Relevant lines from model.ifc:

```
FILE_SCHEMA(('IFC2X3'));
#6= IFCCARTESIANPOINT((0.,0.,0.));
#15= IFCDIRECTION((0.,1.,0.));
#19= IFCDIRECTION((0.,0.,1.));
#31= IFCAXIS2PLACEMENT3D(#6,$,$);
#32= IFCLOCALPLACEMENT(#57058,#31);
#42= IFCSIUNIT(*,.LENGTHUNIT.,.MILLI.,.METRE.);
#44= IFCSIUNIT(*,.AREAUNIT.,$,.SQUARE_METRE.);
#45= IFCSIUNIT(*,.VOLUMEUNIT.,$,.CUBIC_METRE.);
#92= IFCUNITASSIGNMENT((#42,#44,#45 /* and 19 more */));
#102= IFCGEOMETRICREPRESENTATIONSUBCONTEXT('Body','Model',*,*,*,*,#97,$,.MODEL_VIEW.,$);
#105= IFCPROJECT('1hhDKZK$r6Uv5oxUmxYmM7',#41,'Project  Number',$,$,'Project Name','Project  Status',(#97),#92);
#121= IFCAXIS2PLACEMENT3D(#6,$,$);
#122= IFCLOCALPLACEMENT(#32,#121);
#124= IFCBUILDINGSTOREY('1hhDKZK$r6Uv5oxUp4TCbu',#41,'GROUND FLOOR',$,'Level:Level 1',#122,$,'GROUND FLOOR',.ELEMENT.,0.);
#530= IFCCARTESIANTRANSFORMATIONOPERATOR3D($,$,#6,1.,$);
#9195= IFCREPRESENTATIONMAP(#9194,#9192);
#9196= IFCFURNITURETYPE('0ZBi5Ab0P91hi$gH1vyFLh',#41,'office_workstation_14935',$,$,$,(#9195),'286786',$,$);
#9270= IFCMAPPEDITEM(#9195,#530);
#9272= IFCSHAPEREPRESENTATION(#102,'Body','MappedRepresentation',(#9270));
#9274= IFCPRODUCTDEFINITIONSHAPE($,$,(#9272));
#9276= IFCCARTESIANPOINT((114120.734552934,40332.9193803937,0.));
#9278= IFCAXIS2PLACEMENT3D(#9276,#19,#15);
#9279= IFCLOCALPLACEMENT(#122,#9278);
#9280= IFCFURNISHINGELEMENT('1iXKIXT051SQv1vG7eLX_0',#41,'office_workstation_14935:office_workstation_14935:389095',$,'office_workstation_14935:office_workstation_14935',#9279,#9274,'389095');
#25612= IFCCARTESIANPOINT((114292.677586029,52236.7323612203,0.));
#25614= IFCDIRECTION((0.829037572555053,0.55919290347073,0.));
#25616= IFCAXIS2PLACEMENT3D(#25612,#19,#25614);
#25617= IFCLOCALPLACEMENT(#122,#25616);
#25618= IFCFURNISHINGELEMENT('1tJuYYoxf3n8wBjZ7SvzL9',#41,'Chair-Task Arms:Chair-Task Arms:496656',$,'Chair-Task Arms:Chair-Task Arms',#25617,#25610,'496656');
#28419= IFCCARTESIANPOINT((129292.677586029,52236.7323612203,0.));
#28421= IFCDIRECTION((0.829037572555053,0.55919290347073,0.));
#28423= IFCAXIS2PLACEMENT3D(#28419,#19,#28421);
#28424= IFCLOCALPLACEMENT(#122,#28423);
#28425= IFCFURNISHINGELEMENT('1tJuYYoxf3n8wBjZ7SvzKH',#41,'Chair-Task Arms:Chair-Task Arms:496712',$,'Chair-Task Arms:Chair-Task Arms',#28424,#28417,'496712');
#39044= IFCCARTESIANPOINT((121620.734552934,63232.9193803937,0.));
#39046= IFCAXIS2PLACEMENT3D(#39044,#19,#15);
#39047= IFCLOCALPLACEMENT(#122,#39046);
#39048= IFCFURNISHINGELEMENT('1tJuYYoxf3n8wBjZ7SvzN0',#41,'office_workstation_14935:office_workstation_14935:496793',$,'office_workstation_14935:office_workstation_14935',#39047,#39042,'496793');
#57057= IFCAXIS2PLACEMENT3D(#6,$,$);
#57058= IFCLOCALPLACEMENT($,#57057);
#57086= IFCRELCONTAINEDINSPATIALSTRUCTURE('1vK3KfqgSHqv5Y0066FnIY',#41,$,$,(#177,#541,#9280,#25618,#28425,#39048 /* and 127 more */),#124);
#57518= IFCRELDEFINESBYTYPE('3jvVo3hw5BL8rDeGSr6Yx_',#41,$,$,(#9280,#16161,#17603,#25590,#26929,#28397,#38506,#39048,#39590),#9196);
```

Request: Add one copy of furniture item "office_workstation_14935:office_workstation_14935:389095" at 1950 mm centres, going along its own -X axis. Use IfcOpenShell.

```python
import ifcopenshell
import ifcopenshell.api.geometry
import ifcopenshell.api.root
import ifcopenshell.util.element
import ifcopenshell.util.placement
import ifcopenshell.util.unit

model = ifcopenshell.open("model.ifc")
unit_scale = ifcopenshell.util.unit.calculate_unit_scale(model)


def reuse_history(source, copy):
    """copy_class also copies each property set's owner history, people and application; keep the originals."""
    for rel in copy.IsDefinedBy:
        if rel.is_a("IfcRelDefinesByProperties") and (history := rel.RelatingPropertyDefinition.OwnerHistory):
            rel.RelatingPropertyDefinition.OwnerHistory = source.OwnerHistory
            ifcopenshell.util.element.remove_deep2(model, history)


source = model.by_id(9280)
base = ifcopenshell.util.placement.get_local_placement(source.ObjectPlacement)
step = -base[:3, 0] * 1.95 / unit_scale

for i in range(1, 2):
    copy = ifcopenshell.api.root.copy_class(model, product=source)
    copy.Representation = ifcopenshell.util.element.copy_deep(
        model, source.Representation, exclude=["IfcGeometricRepresentationContext", "IfcRepresentationMap"]
    )
    copy.Name = "office_workstation_14935:office_workstation_14935"
    copy.Tag = None
    reuse_history(source, copy)
    matrix = base.copy()
    matrix[:3, 3] += i * step
    print("added at", matrix[:3, 3].round(3) + 0.0)
    ifcopenshell.api.geometry.edit_object_placement(model, product=copy, matrix=matrix, is_si=False)

model.write("model_rev.ifc")
```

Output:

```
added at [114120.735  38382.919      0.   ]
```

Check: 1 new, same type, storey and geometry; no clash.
